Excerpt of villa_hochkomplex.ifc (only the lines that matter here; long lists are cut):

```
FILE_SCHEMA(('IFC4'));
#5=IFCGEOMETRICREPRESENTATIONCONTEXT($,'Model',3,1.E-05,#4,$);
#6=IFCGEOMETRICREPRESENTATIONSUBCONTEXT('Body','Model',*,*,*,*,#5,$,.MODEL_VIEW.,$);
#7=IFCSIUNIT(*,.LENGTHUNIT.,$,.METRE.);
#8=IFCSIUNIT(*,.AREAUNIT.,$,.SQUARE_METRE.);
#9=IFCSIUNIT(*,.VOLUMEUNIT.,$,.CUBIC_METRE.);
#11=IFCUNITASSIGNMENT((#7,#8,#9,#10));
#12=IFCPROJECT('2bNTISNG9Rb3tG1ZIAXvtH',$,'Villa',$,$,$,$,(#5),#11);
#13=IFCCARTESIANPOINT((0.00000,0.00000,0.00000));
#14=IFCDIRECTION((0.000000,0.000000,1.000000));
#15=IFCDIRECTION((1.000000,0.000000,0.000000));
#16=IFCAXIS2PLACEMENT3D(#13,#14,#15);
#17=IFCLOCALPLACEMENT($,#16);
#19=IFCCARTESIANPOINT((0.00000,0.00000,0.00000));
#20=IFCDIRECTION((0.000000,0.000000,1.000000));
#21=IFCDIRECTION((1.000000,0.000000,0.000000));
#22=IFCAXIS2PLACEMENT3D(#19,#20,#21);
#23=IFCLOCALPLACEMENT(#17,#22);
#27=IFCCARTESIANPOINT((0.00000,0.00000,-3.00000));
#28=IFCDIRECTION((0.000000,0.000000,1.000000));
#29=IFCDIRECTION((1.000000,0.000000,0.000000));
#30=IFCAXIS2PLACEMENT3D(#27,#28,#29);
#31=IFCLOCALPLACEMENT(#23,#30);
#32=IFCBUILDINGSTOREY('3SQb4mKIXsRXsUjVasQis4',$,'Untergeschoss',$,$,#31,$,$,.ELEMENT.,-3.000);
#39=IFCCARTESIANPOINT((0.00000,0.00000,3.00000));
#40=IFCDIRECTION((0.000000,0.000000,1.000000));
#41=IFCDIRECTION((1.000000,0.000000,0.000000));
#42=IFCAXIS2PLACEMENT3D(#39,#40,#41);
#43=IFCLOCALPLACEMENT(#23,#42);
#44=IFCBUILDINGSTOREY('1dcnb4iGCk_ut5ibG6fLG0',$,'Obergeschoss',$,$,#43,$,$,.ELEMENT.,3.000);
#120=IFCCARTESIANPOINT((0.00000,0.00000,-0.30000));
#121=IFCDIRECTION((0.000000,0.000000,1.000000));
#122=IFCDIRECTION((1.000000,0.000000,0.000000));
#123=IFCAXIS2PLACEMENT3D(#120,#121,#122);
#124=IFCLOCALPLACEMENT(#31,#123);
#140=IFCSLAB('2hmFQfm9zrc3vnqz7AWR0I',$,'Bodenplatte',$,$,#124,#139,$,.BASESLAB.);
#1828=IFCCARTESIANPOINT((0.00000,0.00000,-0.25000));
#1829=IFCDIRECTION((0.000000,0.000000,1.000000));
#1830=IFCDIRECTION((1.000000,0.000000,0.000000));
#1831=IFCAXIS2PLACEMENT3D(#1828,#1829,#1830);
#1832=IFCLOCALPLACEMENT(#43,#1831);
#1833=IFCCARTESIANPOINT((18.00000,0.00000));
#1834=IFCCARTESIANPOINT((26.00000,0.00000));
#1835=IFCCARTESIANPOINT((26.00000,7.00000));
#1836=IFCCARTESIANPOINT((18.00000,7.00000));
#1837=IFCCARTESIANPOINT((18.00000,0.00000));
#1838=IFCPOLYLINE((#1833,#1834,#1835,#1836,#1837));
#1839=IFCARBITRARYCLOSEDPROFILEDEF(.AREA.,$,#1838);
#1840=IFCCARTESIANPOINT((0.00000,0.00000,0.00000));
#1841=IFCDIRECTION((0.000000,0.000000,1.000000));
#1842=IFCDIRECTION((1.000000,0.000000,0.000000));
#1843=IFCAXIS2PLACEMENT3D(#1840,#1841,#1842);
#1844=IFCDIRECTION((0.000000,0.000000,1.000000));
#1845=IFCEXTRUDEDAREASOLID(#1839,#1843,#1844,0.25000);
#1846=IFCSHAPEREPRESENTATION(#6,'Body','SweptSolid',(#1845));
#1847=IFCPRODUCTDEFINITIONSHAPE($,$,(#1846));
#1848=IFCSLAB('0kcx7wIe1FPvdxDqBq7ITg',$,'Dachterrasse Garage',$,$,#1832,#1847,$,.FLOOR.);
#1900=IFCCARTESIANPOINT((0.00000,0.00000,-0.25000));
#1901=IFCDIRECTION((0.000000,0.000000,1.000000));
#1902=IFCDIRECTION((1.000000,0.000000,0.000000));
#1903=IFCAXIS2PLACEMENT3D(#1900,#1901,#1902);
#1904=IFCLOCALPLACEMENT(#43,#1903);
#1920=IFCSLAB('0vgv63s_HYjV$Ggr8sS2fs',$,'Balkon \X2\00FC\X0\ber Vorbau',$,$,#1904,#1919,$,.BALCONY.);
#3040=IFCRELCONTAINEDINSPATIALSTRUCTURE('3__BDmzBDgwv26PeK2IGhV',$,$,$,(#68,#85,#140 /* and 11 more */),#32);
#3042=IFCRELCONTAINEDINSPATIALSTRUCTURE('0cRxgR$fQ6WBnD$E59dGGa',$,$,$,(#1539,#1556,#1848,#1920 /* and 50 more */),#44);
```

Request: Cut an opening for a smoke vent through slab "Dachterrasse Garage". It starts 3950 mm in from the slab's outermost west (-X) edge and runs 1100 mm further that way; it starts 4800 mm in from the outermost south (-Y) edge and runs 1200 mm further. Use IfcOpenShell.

```python
import numpy as np
import ifcopenshell
import ifcopenshell.api.feature
import ifcopenshell.api.geometry
import ifcopenshell.api.root
import ifcopenshell.geom
import ifcopenshell.util.placement
import ifcopenshell.util.representation
import ifcopenshell.util.shape
import ifcopenshell.util.unit

model = ifcopenshell.open("villa_hochkomplex.ifc")
unit_scale = ifcopenshell.util.unit.calculate_unit_scale(model)
settings = ifcopenshell.geom.settings()


def volume(element):
    """Net volume in cubic metres, openings subtracted."""
    shape = ifcopenshell.geom.create_shape(settings, element)
    return ifcopenshell.util.shape.get_volume(shape.geometry)


slab = model.by_id(1848)
before = volume(slab)

# Extent in the slab's own axes, in metres. The edges named are its -X and -Y sides.
slab_shape = ifcopenshell.geom.create_shape(settings, slab)
vertices = ifcopenshell.util.shape.get_vertices(slab_shape.geometry)
x_min, y_min, bottom = vertices.min(axis=0)
top = vertices[:, 2].max()

opening = ifcopenshell.api.root.create_entity(model, ifc_class="IfcOpeningElement", name="Smoke vent opening", predefined_type="OPENING")
context = ifcopenshell.util.representation.get_context(model, "Model", "Body", "MODEL_VIEW")
width, depth = 1.1, 1.2
outline = [(0.0, 0.0), (width, 0.0), (width, depth), (0.0, depth), (0.0, 0.0)]
# Overshoot both faces by 50 mm so the cut is clean.
shape = ifcopenshell.api.geometry.add_slab_representation(
    model, context=context, depth=top - bottom + 0.1, polyline=outline
)
ifcopenshell.api.geometry.assign_representation(model, product=opening, representation=shape)

matrix = ifcopenshell.util.placement.get_local_placement(slab.ObjectPlacement)
matrix[:, 3] = matrix @ np.append(np.array([x_min + 3.95, y_min + 4.8, bottom - 0.05]) / unit_scale, 1.0)
ifcopenshell.api.geometry.edit_object_placement(model, product=opening, matrix=matrix, is_si=False)
ifcopenshell.api.feature.add_feature(model, feature=opening, element=slab)

after = volume(slab)

print(f"slab volume {before:.3f} -> {after:.3f} m3")

model.write("villa_hochkomplex_updated.ifc")
```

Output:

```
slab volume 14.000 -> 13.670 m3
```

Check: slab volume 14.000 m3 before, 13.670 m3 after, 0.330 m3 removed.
